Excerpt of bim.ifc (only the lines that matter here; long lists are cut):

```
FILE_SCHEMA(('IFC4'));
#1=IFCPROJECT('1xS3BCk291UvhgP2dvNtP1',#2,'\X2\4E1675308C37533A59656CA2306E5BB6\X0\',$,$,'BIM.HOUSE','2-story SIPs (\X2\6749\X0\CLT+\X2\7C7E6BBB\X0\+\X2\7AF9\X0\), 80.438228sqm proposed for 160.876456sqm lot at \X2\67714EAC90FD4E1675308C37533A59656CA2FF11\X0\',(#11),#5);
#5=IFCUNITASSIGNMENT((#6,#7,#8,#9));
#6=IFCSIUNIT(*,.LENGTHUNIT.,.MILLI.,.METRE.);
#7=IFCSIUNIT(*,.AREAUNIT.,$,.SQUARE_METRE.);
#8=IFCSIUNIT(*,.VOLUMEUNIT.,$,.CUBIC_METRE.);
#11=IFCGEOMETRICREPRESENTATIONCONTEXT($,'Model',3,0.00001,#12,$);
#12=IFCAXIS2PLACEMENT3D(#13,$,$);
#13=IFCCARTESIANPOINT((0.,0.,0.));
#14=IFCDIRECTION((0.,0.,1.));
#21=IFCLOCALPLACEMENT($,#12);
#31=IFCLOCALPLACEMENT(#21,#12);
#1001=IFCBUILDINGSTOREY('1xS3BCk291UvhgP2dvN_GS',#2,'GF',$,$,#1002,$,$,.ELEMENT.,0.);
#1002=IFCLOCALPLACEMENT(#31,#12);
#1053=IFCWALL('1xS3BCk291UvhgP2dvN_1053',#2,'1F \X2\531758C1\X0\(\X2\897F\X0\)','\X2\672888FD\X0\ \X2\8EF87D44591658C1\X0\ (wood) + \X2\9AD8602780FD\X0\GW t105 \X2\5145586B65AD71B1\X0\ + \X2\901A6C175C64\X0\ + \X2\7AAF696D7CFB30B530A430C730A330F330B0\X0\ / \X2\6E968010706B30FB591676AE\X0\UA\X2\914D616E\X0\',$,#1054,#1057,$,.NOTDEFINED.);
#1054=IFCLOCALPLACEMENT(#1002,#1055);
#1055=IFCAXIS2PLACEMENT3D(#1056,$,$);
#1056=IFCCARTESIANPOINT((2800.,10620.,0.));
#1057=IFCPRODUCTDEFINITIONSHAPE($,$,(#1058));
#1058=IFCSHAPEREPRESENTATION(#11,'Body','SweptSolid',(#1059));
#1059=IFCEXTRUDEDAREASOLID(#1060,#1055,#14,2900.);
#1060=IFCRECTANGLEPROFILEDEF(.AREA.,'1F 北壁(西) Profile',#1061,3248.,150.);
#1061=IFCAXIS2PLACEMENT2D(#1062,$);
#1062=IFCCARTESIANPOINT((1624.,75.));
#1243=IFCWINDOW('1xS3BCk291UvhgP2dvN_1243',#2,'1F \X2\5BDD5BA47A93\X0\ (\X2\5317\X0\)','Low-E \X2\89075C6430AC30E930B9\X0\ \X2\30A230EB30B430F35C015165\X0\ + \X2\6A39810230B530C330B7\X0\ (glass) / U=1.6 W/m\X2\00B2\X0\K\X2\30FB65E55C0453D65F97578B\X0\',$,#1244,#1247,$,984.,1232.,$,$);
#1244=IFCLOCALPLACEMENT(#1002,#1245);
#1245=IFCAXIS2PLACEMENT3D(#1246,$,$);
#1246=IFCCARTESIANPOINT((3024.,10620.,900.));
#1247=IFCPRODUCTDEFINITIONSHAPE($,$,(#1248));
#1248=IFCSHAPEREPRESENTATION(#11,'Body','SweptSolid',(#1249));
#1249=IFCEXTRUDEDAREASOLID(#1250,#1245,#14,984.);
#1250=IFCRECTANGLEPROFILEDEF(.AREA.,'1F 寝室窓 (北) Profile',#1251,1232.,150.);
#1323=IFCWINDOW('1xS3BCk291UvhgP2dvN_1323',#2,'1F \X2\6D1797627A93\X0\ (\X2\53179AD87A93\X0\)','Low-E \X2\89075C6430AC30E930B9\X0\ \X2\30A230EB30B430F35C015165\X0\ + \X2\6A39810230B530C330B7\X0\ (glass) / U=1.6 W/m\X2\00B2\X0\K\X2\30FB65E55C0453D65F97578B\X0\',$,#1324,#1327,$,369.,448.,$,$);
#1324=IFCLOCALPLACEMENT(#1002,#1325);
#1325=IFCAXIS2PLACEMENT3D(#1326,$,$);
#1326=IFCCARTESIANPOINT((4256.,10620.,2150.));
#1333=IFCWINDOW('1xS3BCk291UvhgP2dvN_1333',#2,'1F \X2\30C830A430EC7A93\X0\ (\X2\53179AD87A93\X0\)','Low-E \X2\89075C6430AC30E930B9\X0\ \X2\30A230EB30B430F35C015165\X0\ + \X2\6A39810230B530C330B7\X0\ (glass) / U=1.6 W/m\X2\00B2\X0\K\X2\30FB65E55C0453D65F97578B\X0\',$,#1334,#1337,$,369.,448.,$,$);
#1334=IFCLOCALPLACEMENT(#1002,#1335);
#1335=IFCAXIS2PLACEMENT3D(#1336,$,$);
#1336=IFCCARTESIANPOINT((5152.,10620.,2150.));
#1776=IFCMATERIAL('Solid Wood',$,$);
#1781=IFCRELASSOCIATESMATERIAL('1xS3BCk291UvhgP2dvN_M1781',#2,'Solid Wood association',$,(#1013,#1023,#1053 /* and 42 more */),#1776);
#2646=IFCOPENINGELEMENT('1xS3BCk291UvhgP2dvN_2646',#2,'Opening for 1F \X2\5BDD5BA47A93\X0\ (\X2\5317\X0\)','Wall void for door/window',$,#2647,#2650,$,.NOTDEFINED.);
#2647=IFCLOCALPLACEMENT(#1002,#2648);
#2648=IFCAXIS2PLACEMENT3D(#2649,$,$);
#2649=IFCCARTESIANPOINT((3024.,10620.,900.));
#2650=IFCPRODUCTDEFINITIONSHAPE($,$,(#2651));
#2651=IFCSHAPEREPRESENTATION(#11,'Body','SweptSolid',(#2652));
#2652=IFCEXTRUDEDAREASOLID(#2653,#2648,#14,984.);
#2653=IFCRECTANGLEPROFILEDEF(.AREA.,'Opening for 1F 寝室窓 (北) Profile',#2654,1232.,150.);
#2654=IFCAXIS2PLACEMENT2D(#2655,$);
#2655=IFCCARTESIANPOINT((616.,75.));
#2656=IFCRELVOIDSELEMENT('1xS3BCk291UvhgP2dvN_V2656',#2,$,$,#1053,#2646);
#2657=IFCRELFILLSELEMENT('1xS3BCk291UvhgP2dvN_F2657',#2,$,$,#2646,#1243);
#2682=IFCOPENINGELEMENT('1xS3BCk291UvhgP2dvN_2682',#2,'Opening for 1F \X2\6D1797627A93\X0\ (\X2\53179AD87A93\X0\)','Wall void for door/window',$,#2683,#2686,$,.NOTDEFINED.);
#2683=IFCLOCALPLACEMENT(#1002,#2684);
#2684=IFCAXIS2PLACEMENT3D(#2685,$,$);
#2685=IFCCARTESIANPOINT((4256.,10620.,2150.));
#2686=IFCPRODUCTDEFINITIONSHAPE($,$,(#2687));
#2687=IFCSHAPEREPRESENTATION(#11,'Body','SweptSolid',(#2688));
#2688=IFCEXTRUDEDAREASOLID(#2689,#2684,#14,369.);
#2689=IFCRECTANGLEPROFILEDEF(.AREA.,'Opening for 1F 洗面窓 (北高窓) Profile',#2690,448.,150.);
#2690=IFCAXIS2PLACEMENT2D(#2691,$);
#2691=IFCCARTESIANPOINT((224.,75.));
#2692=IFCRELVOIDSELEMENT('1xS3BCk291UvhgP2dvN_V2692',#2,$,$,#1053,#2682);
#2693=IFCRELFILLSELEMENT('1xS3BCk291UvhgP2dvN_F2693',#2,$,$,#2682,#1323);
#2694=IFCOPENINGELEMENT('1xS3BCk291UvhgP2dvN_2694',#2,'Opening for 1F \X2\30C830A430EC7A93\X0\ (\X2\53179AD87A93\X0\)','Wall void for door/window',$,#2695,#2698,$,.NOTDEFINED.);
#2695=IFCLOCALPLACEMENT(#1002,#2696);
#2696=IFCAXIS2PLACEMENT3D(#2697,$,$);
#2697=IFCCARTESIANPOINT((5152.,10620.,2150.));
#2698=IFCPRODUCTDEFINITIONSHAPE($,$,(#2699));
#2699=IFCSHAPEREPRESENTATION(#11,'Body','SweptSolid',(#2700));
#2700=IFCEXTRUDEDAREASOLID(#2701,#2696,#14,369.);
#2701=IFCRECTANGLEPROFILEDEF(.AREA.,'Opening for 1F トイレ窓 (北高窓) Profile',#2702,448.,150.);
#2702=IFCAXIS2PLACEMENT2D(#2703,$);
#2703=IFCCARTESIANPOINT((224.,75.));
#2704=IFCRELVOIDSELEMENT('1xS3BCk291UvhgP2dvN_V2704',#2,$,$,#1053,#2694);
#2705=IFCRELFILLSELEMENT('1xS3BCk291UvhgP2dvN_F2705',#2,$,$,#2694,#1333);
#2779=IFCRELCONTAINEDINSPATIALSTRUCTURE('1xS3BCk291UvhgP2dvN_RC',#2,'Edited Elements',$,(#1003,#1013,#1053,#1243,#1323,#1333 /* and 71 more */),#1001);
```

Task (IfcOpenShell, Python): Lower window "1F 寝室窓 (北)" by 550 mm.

```python
import numpy as np
import ifcopenshell
import ifcopenshell.api.geometry
import ifcopenshell.util.placement
import ifcopenshell.util.unit

model = ifcopenshell.open("bim.ifc")
unit_scale = ifcopenshell.util.unit.calculate_unit_scale(model)

window = model.by_guid("1xS3BCk291UvhgP2dvN_1243")
opening = window.FillsVoids[0].RelatingOpeningElement
dz = -0.55 / unit_scale

shift = np.array([0.0, 0.0, dz])
# The window is not placed relative to its opening, so move both.
for product in (opening, window):
    matrix = ifcopenshell.util.placement.get_local_placement(product.ObjectPlacement)
    matrix[:3, 3] += shift
    ifcopenshell.api.geometry.edit_object_placement(model, product=product, matrix=matrix, is_si=False)

print(f"moved by {dz * unit_scale:+.3f} m")

model.write("bim_updated.ifc")
```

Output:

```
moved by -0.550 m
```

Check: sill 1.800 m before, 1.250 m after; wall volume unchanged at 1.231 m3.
